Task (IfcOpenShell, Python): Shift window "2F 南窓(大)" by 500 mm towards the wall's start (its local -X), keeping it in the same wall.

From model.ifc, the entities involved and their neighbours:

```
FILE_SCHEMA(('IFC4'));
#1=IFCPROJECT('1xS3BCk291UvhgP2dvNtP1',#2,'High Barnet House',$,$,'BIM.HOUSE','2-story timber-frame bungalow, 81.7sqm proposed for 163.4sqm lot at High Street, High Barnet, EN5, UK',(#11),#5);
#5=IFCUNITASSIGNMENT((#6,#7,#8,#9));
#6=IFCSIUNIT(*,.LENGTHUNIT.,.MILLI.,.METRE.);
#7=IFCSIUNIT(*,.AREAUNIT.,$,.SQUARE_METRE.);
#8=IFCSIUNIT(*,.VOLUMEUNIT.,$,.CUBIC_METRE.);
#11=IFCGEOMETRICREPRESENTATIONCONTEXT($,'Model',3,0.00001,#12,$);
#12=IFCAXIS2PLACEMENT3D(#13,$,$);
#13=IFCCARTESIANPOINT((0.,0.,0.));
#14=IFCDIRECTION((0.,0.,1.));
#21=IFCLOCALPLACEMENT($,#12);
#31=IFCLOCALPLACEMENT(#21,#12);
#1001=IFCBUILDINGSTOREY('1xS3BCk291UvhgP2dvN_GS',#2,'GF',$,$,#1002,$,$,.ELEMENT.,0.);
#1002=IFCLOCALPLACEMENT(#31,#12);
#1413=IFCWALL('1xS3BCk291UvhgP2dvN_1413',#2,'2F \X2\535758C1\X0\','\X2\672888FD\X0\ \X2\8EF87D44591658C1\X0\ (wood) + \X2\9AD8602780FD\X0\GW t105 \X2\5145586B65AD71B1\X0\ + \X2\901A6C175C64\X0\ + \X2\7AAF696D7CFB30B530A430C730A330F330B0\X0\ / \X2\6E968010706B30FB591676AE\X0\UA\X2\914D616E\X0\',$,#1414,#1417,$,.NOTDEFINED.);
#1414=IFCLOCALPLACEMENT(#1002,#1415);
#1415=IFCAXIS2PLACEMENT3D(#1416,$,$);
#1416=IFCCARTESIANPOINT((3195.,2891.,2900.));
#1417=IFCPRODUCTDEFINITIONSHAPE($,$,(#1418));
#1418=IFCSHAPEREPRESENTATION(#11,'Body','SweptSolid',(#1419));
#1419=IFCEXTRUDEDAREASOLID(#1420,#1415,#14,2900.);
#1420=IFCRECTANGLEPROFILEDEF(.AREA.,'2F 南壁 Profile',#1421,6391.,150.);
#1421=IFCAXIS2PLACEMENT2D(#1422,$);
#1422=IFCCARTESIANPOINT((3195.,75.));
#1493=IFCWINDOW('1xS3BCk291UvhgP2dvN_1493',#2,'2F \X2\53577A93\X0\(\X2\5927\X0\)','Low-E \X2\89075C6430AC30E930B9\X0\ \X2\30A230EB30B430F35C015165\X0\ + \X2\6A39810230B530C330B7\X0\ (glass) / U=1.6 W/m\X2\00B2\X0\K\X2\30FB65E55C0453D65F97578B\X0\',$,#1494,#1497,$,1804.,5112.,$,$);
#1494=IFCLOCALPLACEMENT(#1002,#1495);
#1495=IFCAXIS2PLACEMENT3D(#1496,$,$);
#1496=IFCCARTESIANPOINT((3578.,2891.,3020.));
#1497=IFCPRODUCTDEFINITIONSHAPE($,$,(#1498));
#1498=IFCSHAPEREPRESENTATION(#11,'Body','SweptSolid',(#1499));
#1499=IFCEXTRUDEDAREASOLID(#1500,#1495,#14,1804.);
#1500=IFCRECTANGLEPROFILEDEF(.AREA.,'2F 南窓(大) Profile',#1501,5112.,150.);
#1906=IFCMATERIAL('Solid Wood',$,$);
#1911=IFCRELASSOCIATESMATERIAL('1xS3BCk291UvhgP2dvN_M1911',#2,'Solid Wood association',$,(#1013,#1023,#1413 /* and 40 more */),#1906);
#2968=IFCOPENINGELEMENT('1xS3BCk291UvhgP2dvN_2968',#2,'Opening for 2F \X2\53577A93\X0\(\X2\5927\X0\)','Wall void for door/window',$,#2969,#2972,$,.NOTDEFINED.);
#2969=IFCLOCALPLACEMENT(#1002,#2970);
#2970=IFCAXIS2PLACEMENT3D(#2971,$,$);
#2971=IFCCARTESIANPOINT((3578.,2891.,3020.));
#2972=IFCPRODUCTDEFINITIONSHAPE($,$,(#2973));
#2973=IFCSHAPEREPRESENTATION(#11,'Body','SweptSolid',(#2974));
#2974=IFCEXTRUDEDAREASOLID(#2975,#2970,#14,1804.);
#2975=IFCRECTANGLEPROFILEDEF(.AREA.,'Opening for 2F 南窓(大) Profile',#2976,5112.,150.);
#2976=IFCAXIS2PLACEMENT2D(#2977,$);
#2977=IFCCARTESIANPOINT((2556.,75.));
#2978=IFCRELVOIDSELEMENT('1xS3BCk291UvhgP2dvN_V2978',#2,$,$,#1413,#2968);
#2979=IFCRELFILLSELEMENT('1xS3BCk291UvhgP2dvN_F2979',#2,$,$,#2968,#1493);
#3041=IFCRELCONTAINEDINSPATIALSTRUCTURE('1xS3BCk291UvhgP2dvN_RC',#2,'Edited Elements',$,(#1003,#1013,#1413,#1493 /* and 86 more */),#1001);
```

```python
import ifcopenshell
import ifcopenshell.api.geometry
import ifcopenshell.util.placement

model = ifcopenshell.open("model.ifc")

window = model.by_guid("1xS3BCk291UvhgP2dvN_1493")
opening = window.FillsVoids[0].RelatingOpeningElement
wall = opening.VoidsElements[0].RelatingBuildingElement

wall_matrix = ifcopenshell.util.placement.get_local_placement(wall.ObjectPlacement)
shift = wall_matrix[:3, 0] * -500.0
before = ifcopenshell.util.placement.get_local_placement(window.ObjectPlacement)[:3, 3].copy()

# The window is not placed relative to its opening, so move both.
for product in (opening, window):
    matrix = ifcopenshell.util.placement.get_local_placement(product.ObjectPlacement)
    matrix[:3, 3] += shift
    ifcopenshell.api.geometry.edit_object_placement(model, product=product, matrix=matrix, is_si=False)

after = ifcopenshell.util.placement.get_local_placement(window.ObjectPlacement)[:3, 3]
print("window moved by", (after - before).round(3) + 0.0)

model.write("model_edited.ifc")
```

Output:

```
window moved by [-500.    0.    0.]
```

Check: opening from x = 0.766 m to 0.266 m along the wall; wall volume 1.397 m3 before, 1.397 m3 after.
